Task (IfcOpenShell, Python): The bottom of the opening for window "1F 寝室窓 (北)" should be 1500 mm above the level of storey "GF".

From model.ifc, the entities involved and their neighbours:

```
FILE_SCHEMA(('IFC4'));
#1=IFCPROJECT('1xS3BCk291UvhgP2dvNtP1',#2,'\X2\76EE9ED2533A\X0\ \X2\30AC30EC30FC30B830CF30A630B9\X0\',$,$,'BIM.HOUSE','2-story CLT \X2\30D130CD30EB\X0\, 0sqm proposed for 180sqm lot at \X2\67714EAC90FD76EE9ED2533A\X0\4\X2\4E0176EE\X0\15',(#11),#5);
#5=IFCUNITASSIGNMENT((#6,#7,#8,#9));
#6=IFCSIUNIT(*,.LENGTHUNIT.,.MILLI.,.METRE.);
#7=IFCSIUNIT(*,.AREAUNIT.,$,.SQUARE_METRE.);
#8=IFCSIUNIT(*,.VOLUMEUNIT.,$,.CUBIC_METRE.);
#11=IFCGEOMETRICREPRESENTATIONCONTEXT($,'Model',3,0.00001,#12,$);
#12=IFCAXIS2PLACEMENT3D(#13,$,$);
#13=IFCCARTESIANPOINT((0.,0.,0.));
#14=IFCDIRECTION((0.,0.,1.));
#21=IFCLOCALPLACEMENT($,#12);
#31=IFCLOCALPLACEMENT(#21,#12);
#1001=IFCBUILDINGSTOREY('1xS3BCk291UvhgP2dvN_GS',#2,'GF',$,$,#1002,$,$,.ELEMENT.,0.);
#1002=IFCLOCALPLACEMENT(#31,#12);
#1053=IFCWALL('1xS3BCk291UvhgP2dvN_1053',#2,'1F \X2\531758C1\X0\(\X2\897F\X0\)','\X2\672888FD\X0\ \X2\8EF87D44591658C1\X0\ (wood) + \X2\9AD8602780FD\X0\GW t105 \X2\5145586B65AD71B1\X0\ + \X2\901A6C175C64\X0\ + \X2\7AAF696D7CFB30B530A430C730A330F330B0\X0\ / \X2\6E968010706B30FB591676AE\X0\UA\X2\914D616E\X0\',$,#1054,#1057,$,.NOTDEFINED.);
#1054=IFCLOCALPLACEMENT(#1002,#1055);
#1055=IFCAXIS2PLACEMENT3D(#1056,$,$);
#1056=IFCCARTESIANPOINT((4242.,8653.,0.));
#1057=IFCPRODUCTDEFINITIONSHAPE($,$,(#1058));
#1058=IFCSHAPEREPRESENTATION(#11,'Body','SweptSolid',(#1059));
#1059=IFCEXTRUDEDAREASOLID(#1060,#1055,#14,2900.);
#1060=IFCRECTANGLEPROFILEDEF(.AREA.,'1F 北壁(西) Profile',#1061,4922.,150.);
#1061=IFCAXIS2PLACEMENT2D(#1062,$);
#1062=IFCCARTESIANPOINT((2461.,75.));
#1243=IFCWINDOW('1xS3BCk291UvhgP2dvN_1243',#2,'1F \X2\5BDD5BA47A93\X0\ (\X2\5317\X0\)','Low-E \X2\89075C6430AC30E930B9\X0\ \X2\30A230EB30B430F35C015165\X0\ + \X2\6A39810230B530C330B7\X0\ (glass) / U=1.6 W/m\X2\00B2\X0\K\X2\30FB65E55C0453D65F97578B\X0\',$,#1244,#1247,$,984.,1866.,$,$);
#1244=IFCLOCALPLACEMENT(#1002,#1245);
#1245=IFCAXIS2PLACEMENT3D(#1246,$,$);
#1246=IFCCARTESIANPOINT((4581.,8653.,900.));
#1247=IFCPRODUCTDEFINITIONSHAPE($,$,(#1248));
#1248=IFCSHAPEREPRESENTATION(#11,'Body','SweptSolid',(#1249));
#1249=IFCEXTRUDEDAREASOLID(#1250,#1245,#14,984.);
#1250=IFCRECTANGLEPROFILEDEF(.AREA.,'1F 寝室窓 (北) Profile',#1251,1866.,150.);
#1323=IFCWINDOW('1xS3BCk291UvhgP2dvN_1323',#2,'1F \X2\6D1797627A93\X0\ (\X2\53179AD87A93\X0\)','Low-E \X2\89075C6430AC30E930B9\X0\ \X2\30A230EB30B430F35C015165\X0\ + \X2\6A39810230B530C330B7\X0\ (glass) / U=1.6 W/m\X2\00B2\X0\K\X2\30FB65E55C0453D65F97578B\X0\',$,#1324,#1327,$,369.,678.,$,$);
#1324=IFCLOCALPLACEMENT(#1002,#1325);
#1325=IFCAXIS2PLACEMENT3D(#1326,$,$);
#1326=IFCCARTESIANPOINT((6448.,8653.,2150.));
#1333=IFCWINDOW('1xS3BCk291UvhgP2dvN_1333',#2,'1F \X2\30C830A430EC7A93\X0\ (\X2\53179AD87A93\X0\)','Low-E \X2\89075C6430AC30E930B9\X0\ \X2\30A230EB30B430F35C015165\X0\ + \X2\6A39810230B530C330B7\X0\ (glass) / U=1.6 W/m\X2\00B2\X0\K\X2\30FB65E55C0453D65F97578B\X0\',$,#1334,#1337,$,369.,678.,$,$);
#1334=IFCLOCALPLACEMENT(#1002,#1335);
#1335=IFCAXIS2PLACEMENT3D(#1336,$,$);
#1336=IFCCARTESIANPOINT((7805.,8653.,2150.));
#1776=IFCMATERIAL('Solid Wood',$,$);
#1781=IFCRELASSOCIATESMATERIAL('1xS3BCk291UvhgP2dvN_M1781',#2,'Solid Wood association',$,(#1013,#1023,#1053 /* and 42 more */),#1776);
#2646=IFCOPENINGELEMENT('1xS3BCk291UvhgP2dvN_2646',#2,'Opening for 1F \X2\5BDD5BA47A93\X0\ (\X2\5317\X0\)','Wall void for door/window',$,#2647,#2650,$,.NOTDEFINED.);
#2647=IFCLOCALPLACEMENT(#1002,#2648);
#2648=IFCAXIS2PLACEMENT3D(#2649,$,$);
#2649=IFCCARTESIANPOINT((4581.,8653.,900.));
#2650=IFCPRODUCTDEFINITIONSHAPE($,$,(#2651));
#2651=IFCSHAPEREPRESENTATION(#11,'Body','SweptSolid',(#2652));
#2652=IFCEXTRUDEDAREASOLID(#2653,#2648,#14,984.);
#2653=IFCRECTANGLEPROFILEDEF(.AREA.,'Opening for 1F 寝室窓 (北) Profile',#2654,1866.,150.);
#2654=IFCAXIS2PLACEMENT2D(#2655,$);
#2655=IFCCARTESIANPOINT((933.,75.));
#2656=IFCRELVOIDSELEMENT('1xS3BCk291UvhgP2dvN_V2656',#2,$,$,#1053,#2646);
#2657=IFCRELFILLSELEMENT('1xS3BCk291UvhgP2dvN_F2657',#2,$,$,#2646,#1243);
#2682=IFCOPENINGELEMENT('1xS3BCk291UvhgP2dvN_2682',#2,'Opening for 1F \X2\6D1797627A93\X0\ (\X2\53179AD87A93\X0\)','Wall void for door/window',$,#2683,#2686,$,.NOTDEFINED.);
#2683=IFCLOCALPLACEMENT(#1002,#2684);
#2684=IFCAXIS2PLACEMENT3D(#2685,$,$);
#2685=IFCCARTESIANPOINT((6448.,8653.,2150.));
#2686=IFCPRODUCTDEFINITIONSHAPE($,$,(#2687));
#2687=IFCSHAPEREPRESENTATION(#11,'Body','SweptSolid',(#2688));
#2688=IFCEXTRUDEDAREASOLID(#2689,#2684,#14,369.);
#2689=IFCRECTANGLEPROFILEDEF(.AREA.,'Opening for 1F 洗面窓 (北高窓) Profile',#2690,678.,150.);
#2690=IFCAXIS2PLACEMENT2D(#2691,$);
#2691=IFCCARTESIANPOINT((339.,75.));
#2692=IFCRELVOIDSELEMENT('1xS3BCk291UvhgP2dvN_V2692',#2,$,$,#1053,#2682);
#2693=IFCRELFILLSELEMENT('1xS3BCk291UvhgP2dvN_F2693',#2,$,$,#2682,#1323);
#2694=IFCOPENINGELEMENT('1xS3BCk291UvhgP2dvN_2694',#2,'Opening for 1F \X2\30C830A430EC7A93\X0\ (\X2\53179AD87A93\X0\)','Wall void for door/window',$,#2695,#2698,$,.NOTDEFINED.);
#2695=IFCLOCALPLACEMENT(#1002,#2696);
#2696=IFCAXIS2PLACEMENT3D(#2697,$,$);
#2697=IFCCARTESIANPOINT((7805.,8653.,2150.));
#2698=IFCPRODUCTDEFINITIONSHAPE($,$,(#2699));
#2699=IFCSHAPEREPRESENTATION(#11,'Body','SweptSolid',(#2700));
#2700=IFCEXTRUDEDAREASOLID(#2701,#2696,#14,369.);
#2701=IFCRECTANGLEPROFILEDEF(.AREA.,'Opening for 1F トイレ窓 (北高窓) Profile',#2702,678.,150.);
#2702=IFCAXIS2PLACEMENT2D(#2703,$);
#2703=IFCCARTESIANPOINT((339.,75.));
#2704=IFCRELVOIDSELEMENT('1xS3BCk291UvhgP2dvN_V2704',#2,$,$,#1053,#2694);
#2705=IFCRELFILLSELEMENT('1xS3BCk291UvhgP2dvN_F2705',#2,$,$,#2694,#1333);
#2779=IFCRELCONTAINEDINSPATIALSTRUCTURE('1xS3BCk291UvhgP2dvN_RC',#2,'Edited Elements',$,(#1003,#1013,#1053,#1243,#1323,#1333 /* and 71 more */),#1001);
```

```python
import numpy as np
import ifcopenshell
import ifcopenshell.api.geometry
import ifcopenshell.geom
import ifcopenshell.util.element
import ifcopenshell.util.placement
import ifcopenshell.util.shape
import ifcopenshell.util.unit

model = ifcopenshell.open("model.ifc")
unit_scale = ifcopenshell.util.unit.calculate_unit_scale(model)

window = model.by_id(1243)
opening = window.FillsVoids[0].RelatingOpeningElement
storey = ifcopenshell.util.element.get_container(window, ifc_class="IfcBuildingStorey")
level = ifcopenshell.util.placement.get_local_placement(storey.ObjectPlacement)[2, 3]

# The opening's origin need not be at the sill, so measure its lowest point.
shape = ifcopenshell.geom.create_shape(ifcopenshell.geom.settings(), opening)
bottom = ifcopenshell.util.shape.get_shape_bottom_elevation(shape, shape.geometry) / unit_scale
dz = level + 1.5 / unit_scale - bottom

shift = np.array([0.0, 0.0, dz])
# The window is not placed relative to its opening, so move both.
for product in (opening, window):
    matrix = ifcopenshell.util.placement.get_local_placement(product.ObjectPlacement)
    matrix[:3, 3] += shift
    ifcopenshell.api.geometry.edit_object_placement(model, product=product, matrix=matrix, is_si=False)

print(f"moved by {dz * unit_scale:+.3f} m")

model.write("model-out.ifc")
```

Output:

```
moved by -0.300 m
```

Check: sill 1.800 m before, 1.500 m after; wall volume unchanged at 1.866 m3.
